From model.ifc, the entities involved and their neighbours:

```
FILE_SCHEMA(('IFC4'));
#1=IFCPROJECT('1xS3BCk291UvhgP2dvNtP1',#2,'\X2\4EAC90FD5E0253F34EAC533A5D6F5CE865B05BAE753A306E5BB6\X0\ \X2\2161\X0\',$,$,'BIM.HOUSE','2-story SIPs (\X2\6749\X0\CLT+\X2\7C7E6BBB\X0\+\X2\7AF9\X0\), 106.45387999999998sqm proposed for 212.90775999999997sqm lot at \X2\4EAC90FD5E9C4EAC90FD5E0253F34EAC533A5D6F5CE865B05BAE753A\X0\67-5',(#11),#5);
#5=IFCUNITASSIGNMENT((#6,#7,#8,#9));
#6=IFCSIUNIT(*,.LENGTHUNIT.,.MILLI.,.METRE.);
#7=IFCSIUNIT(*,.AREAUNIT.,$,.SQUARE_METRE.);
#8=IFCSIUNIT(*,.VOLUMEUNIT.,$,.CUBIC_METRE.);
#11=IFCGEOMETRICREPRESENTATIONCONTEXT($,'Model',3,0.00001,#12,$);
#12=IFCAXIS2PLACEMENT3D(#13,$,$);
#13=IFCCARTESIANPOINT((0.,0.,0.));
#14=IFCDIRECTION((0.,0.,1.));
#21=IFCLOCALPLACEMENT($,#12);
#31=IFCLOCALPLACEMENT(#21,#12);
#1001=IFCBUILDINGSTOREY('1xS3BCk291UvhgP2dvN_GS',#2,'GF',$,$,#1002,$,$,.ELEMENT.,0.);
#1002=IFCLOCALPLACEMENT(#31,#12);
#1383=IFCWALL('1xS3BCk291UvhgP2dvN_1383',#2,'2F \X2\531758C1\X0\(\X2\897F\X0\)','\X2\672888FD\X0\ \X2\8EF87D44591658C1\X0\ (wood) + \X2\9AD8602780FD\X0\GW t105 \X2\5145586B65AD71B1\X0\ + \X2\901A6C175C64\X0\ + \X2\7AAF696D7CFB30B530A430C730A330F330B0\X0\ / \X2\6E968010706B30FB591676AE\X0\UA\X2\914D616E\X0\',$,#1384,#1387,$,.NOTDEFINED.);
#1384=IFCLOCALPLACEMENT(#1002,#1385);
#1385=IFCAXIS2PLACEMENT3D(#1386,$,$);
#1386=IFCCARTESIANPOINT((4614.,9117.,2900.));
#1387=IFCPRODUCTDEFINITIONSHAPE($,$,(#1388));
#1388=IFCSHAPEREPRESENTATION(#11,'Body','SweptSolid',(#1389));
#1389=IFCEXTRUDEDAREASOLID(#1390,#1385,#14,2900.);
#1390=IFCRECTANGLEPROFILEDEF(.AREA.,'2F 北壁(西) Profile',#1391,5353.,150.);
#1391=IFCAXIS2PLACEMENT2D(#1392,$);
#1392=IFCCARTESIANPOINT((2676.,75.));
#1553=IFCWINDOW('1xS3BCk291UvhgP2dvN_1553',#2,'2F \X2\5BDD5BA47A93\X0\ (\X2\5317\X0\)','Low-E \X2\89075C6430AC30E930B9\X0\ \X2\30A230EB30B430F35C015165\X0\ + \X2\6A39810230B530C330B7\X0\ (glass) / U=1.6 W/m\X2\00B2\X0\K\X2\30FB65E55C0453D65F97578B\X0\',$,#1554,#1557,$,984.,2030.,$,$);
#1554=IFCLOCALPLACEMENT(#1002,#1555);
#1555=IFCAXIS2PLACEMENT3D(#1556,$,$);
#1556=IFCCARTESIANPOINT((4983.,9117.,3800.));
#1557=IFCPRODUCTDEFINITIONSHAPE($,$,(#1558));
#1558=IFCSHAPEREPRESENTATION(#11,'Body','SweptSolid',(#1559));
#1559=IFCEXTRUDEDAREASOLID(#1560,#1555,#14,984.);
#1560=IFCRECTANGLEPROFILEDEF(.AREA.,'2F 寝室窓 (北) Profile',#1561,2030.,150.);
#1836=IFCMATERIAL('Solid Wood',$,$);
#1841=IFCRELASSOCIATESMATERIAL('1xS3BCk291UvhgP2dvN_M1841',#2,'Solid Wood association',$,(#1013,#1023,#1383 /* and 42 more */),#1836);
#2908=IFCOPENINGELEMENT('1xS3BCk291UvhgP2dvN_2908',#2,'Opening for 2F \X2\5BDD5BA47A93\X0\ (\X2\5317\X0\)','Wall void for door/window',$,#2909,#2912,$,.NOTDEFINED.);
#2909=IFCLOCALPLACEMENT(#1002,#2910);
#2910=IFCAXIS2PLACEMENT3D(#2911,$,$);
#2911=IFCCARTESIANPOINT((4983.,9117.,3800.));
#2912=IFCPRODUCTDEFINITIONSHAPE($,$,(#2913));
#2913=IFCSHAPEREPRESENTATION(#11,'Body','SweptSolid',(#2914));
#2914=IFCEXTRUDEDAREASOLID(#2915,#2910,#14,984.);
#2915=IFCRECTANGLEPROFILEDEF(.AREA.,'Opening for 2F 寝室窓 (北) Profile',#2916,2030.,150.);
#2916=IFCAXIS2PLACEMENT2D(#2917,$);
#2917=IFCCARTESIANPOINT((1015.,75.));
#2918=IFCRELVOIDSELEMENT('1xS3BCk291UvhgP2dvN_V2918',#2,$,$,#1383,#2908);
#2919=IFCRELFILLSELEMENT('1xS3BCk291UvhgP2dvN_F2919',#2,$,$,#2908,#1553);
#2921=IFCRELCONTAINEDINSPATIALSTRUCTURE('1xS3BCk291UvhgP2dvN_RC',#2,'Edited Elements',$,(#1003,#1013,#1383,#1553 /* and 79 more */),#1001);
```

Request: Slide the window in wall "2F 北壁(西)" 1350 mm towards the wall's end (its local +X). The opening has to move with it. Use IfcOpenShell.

```python
import ifcopenshell
import ifcopenshell.api.geometry
import ifcopenshell.util.placement

model = ifcopenshell.open("model.ifc")

window = model.by_guid("1xS3BCk291UvhgP2dvN_1553")
opening = window.FillsVoids[0].RelatingOpeningElement
wall = opening.VoidsElements[0].RelatingBuildingElement

wall_matrix = ifcopenshell.util.placement.get_local_placement(wall.ObjectPlacement)
shift = wall_matrix[:3, 0] * 1350.0
before = ifcopenshell.util.placement.get_local_placement(window.ObjectPlacement)[:3, 3].copy()

# The window is not placed relative to its opening, so move both.
for product in (opening, window):
    matrix = ifcopenshell.util.placement.get_local_placement(product.ObjectPlacement)
    matrix[:3, 3] += shift
    ifcopenshell.api.geometry.edit_object_placement(model, product=product, matrix=matrix, is_si=False)

after = ifcopenshell.util.placement.get_local_placement(window.ObjectPlacement)[:3, 3]
print("window moved by", (after - before).round(3) + 0.0)

model.write("model_updated.ifc")
```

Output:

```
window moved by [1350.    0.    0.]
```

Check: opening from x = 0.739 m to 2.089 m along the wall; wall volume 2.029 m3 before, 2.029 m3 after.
